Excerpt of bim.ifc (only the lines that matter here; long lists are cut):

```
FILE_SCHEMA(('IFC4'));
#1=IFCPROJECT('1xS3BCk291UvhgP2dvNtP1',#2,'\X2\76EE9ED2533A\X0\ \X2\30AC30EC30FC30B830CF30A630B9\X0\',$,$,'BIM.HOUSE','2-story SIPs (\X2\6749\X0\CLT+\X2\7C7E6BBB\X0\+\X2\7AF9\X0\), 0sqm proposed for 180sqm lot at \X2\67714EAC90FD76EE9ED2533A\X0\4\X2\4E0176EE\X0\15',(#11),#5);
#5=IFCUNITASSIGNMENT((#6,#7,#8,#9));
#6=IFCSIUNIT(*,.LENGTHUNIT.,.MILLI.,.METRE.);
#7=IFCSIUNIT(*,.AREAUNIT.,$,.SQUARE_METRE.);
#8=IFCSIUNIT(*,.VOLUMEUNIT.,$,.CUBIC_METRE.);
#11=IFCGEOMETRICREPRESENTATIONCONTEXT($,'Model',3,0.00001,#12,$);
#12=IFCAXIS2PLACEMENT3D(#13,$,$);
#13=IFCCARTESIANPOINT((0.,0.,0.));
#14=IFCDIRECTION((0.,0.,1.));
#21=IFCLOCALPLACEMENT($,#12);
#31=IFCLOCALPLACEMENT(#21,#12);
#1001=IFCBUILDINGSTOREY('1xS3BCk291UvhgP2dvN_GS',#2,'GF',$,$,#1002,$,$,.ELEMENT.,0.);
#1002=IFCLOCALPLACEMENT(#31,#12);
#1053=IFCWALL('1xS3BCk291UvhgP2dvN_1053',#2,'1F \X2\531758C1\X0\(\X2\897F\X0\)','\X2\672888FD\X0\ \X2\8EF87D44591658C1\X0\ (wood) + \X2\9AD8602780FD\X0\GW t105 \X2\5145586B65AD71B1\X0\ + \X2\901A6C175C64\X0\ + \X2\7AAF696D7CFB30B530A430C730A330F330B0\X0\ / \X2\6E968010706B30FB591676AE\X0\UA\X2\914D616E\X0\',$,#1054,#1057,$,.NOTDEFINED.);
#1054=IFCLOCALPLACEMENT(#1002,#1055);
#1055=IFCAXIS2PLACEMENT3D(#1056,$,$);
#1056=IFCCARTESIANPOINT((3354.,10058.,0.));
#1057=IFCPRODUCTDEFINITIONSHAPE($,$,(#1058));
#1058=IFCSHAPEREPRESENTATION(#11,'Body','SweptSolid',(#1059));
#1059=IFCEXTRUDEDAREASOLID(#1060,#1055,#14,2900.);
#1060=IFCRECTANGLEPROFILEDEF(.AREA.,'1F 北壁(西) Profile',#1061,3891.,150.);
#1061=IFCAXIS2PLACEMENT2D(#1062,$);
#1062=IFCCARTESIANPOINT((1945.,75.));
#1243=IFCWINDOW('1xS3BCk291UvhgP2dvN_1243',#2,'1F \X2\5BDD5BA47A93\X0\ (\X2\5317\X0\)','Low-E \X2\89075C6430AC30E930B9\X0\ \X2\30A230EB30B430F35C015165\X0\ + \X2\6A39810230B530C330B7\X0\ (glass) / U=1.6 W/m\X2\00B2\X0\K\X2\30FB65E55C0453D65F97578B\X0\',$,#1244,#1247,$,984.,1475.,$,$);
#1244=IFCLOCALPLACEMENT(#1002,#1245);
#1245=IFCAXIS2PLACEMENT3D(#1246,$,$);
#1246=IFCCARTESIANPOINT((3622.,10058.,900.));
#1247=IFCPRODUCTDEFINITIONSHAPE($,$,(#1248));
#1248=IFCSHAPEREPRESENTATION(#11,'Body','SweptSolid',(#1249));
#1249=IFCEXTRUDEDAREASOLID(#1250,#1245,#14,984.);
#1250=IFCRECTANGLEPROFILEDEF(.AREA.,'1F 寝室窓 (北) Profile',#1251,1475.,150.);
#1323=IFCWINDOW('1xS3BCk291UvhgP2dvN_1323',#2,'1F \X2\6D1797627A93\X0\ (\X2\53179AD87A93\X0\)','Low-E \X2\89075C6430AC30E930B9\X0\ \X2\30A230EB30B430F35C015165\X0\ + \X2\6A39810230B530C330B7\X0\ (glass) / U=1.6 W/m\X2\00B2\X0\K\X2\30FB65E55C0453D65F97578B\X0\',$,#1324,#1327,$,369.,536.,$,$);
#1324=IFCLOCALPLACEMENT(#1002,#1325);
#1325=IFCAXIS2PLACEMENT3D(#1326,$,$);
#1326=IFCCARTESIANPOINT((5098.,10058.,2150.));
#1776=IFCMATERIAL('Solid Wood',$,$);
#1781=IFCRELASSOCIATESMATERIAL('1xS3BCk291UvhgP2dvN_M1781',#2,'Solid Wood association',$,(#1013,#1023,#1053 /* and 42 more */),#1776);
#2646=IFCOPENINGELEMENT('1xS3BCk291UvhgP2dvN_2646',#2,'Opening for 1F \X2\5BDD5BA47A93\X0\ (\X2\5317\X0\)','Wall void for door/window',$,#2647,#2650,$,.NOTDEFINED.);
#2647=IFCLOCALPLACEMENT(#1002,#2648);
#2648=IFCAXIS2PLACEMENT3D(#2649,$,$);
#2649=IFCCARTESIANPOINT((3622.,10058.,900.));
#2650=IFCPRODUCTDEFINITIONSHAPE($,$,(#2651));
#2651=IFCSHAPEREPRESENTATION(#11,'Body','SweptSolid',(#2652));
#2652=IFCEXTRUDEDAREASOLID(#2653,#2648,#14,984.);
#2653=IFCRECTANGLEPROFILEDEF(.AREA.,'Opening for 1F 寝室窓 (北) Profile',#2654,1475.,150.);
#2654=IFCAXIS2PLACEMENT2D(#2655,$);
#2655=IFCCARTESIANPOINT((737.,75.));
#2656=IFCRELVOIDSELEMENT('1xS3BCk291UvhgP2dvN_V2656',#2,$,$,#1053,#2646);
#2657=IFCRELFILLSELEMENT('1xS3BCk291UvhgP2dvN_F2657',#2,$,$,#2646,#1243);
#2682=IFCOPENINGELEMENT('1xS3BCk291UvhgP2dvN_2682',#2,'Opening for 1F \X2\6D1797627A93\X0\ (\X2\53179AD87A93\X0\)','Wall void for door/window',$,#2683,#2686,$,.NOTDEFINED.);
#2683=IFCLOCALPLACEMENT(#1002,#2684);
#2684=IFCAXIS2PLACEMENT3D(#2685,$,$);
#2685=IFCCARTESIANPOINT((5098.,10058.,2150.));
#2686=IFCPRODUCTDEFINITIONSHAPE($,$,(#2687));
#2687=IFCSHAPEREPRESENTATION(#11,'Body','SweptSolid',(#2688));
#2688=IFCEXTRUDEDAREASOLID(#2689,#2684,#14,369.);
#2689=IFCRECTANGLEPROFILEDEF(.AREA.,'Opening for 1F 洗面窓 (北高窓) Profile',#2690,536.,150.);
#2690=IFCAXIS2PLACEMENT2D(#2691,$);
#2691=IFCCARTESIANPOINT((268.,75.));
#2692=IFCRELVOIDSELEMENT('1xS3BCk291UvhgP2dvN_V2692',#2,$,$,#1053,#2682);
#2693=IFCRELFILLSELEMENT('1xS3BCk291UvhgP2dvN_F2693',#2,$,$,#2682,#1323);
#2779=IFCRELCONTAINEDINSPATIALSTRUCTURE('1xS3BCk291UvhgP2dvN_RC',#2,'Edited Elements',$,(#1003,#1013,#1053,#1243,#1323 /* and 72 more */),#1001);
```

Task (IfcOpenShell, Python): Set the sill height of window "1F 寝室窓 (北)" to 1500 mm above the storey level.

```python
import numpy as np
import ifcopenshell
import ifcopenshell.api.geometry
import ifcopenshell.geom
import ifcopenshell.util.element
import ifcopenshell.util.placement
import ifcopenshell.util.shape
import ifcopenshell.util.unit

model = ifcopenshell.open("bim.ifc")
unit_scale = ifcopenshell.util.unit.calculate_unit_scale(model)

window = model.by_guid("1xS3BCk291UvhgP2dvN_1243")
opening = window.FillsVoids[0].RelatingOpeningElement
storey = ifcopenshell.util.element.get_container(window, ifc_class="IfcBuildingStorey")
level = ifcopenshell.util.placement.get_local_placement(storey.ObjectPlacement)[2, 3]

# The opening's origin need not be at the sill, so measure its lowest point.
shape = ifcopenshell.geom.create_shape(ifcopenshell.geom.settings(), opening)
bottom = ifcopenshell.util.shape.get_shape_bottom_elevation(shape, shape.geometry) / unit_scale
dz = level + 1.5 / unit_scale - bottom

shift = np.array([0.0, 0.0, dz])
# The window is not placed relative to its opening, so move both.
for product in (opening, window):
    matrix = ifcopenshell.util.placement.get_local_placement(product.ObjectPlacement)
    matrix[:3, 3] += shift
    ifcopenshell.api.geometry.edit_object_placement(model, product=product, matrix=matrix, is_si=False)

print(f"moved by {dz * unit_scale:+.3f} m")

model.write("bim_rev.ifc")
```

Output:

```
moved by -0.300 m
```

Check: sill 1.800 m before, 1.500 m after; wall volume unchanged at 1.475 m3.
